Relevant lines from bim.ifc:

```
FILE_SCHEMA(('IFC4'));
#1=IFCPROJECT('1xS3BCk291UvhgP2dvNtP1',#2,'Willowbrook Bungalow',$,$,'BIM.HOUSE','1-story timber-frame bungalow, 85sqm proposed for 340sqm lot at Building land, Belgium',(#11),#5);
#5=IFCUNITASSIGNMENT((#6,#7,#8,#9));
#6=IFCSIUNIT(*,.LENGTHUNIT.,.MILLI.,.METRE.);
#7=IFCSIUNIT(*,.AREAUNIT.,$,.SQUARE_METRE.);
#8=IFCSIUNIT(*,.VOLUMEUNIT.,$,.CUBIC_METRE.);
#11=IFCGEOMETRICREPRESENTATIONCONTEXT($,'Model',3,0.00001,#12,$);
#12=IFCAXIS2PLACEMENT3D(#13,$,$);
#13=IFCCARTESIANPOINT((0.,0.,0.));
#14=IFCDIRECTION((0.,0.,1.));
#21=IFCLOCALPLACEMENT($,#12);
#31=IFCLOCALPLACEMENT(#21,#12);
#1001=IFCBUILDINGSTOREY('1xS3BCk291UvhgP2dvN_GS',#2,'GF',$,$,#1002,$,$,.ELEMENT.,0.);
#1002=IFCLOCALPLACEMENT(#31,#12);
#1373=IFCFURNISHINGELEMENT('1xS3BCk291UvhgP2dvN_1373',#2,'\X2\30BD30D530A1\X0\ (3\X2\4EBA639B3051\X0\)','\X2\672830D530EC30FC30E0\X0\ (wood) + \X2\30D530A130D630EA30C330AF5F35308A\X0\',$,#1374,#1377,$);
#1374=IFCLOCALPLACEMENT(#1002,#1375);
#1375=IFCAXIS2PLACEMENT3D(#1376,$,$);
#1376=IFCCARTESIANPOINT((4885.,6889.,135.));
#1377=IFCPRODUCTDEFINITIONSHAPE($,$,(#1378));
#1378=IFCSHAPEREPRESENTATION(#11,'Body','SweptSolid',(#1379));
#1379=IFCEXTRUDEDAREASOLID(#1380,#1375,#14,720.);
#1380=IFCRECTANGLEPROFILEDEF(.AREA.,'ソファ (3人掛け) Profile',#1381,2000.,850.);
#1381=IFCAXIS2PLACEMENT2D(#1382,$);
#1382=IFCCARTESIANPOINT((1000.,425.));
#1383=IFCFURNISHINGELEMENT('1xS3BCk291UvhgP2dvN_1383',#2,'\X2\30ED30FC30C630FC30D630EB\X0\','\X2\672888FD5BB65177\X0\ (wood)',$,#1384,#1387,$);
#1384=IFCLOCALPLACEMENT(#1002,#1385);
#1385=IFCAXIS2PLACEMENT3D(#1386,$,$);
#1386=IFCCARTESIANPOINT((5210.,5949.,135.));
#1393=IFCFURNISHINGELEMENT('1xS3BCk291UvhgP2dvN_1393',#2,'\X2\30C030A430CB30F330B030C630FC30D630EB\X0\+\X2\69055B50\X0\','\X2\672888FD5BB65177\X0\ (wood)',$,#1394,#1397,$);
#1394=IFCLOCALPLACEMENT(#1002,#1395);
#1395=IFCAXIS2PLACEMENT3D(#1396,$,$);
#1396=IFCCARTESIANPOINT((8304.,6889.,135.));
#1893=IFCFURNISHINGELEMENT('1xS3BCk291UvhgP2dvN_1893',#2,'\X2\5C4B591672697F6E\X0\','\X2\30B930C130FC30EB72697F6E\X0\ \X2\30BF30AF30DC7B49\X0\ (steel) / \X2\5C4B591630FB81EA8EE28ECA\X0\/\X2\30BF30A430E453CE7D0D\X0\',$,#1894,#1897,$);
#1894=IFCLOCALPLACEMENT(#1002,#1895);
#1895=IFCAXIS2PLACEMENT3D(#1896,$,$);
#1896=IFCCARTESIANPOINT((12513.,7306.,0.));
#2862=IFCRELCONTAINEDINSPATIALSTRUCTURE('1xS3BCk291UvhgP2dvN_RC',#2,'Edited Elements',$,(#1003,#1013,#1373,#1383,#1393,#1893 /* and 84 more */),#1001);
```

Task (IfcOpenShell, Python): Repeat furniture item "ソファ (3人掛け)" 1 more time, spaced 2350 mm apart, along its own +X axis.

```python
import ifcopenshell
import ifcopenshell.api.geometry
import ifcopenshell.api.root
import ifcopenshell.util.element
import ifcopenshell.util.placement

model = ifcopenshell.open("bim.ifc")


def reuse_history(source, copy):
    """copy_class also copies each property set's owner history, people and application; keep the originals."""
    for rel in copy.IsDefinedBy:
        if rel.is_a("IfcRelDefinesByProperties") and (history := rel.RelatingPropertyDefinition.OwnerHistory):
            rel.RelatingPropertyDefinition.OwnerHistory = source.OwnerHistory
            ifcopenshell.util.element.remove_deep2(model, history)


source = model.by_id(1373)
base = ifcopenshell.util.placement.get_local_placement(source.ObjectPlacement)
step = base[:3, 0] * 2350.0

for i in range(1, 2):
    copy = ifcopenshell.api.root.copy_class(model, product=source)
    copy.Representation = ifcopenshell.util.element.copy_deep(
        model, source.Representation, exclude=["IfcGeometricRepresentationContext", "IfcRepresentationMap"]
    )
    reuse_history(source, copy)
    matrix = base.copy()
    matrix[:3, 3] += i * step
    print("added at", matrix[:3, 3].round(3) + 0.0)
    ifcopenshell.api.geometry.edit_object_placement(model, product=copy, matrix=matrix, is_si=False)

model.write("bim_updated.ifc")
```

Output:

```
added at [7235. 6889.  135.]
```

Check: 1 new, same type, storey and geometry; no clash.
